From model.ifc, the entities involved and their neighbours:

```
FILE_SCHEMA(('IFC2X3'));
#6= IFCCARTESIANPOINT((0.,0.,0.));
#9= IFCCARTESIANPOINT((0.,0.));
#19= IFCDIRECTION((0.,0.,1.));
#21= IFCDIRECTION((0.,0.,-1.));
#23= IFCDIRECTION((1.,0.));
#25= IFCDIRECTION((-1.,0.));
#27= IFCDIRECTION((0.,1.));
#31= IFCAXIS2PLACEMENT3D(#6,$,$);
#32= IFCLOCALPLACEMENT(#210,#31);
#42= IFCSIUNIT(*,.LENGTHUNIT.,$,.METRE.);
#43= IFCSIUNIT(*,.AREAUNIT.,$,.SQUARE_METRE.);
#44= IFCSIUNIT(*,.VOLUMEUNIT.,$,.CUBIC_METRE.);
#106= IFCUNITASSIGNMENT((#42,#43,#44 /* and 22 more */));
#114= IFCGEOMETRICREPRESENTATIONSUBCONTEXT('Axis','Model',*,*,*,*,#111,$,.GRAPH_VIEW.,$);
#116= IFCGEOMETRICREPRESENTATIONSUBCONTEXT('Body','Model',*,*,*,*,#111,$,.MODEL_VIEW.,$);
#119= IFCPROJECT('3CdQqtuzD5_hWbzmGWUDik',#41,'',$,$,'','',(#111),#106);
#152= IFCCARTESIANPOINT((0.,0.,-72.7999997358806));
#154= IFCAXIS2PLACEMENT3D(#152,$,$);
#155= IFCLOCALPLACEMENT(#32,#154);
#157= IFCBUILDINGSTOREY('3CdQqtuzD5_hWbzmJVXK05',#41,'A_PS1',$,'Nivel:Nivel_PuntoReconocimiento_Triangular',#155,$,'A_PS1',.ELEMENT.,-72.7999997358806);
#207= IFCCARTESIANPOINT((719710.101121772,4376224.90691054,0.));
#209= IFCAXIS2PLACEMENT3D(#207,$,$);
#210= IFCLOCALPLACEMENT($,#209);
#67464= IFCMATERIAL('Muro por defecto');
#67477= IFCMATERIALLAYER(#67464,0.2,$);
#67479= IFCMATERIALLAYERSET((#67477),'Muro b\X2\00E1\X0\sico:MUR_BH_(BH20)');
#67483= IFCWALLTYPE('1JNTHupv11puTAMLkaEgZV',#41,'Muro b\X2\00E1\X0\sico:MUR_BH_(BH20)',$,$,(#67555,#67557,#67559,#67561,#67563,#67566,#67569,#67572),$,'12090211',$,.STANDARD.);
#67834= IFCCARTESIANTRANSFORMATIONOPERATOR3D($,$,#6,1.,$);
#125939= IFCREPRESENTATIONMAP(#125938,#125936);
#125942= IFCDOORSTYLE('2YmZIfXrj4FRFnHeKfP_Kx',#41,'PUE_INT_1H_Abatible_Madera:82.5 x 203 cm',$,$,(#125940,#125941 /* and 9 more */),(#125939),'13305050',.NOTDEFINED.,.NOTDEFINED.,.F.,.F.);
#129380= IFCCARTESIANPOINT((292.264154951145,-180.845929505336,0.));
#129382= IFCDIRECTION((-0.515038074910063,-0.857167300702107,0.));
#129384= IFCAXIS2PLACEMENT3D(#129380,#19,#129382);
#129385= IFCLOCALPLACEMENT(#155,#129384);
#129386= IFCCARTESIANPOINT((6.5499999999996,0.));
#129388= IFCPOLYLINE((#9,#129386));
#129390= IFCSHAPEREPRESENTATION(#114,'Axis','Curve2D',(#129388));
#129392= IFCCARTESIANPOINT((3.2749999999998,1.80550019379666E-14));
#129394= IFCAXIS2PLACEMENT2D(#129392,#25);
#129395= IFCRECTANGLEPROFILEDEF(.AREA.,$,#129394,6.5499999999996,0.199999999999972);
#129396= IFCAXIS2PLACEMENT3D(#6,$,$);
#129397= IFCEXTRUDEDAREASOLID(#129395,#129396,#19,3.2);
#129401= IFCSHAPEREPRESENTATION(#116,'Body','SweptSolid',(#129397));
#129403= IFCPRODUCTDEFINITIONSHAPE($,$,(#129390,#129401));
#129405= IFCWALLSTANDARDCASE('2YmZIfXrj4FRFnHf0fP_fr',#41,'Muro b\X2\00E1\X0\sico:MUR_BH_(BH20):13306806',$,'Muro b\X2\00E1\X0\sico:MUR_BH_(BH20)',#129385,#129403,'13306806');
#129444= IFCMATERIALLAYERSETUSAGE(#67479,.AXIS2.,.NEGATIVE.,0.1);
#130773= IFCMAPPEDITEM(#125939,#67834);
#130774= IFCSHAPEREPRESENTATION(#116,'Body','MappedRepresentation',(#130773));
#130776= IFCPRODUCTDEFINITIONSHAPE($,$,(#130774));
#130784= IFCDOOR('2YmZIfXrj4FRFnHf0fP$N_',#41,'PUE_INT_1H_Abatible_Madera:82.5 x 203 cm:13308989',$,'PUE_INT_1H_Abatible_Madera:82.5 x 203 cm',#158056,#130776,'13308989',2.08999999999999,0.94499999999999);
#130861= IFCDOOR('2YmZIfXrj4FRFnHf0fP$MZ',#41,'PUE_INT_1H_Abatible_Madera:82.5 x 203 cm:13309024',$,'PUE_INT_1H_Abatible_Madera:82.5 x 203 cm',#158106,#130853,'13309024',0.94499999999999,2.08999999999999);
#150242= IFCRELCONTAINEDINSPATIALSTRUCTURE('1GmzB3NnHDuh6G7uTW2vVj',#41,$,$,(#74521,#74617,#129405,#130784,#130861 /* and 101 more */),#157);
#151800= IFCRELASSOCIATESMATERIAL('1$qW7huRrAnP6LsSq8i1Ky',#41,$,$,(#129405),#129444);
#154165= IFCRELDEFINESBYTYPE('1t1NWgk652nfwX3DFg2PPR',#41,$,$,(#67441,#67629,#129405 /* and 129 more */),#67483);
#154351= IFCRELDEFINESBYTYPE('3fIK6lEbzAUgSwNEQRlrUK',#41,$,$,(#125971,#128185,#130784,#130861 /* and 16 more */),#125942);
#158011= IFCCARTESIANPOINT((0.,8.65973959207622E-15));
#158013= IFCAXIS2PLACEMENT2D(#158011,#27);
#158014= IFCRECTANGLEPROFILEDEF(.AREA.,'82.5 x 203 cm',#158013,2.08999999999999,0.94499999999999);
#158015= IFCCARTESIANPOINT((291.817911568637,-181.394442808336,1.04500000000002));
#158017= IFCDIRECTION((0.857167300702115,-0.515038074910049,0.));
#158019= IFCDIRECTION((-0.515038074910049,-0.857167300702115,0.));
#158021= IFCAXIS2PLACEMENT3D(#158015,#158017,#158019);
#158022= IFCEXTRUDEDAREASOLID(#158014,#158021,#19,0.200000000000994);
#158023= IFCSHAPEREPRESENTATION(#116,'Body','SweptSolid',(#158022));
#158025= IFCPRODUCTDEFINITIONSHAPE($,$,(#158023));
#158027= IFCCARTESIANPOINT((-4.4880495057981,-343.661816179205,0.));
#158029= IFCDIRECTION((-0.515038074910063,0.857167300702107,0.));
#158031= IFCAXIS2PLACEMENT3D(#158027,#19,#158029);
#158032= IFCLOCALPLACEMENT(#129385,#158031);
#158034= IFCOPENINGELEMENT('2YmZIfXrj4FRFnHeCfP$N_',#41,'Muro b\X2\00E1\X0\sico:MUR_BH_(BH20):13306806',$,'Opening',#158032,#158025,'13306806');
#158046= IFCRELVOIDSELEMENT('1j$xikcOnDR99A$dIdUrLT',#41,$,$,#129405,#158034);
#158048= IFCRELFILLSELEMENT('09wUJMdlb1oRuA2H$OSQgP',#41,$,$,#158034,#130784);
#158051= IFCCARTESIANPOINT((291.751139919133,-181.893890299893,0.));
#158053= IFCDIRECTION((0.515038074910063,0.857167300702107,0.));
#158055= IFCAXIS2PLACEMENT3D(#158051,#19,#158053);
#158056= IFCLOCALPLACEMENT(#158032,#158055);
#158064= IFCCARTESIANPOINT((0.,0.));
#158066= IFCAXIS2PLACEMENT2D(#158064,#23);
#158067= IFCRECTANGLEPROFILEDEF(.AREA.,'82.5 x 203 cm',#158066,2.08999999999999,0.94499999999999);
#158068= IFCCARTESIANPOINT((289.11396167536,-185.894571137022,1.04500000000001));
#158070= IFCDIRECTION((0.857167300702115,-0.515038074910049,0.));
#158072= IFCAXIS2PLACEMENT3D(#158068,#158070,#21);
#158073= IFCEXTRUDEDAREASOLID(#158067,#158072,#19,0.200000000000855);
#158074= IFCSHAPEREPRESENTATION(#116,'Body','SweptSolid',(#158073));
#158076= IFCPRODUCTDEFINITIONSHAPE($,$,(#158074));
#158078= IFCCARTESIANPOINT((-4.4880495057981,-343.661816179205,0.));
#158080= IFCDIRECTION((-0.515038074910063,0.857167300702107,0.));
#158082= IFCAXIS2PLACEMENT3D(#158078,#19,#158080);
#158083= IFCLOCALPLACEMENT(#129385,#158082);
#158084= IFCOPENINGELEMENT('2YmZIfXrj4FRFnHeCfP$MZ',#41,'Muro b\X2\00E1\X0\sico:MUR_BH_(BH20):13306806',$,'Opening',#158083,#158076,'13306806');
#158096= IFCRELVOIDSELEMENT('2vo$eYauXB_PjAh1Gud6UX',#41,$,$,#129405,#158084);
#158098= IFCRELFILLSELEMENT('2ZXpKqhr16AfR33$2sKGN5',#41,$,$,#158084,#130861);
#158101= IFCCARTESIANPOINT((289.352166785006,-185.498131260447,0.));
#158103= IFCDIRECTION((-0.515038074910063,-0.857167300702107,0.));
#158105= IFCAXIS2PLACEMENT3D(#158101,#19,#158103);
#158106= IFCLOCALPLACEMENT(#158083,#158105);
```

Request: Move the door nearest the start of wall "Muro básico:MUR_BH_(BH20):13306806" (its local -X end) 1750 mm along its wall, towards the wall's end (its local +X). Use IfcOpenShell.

```python
import ifcopenshell
import ifcopenshell.api.geometry
import ifcopenshell.util.placement

model = ifcopenshell.open("model.ifc")

door = model.by_id(130784)
opening = door.FillsVoids[0].RelatingOpeningElement
wall = opening.VoidsElements[0].RelatingBuildingElement

wall_matrix = ifcopenshell.util.placement.get_local_placement(wall.ObjectPlacement)
shift = wall_matrix[:3, 0] * 1.75
before = ifcopenshell.util.placement.get_local_placement(door.ObjectPlacement)[:3, 3].copy()

# The door is placed relative to its opening, so it follows when the opening moves.
matrix = ifcopenshell.util.placement.get_local_placement(opening.ObjectPlacement)
matrix[:3, 3] += shift
ifcopenshell.api.geometry.edit_object_placement(
    model, product=opening, matrix=matrix, is_si=False, should_transform_children=True
)

after = ifcopenshell.util.placement.get_local_placement(door.ObjectPlacement)[:3, 3]
print("door moved by", (after - before).round(3) + 0.0)

model.write("model-out.ifc")
```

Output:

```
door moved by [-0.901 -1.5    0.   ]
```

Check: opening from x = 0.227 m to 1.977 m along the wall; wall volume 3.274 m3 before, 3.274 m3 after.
